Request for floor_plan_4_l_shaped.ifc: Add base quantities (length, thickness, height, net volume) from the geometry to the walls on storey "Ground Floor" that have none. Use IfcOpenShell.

First a look at what the model holds.

```python
import ifcopenshell
import ifcopenshell.util.element
import ifcopenshell.util.unit

model = ifcopenshell.open("floor_plan_4_l_shaped.ifc")
print(model.schema)
for unit_type in ("LENGTHUNIT", "AREAUNIT", "VOLUMEUNIT"):
    print(unit_type, ifcopenshell.util.unit.calculate_unit_scale(model, unit_type))
storey = next(s for s in model.by_type("IfcBuildingStorey") if s.Name == "Ground Floor")
walls = [e for e in ifcopenshell.util.element.get_decomposition(storey) if e.is_a("IfcWall")]
for e in sorted(walls, key=lambda e: e.id()):
    print(e.id(), e.is_a(), e.Name, list(ifcopenshell.util.element.get_psets(e, qtos_only=True)), sep=" | ")
```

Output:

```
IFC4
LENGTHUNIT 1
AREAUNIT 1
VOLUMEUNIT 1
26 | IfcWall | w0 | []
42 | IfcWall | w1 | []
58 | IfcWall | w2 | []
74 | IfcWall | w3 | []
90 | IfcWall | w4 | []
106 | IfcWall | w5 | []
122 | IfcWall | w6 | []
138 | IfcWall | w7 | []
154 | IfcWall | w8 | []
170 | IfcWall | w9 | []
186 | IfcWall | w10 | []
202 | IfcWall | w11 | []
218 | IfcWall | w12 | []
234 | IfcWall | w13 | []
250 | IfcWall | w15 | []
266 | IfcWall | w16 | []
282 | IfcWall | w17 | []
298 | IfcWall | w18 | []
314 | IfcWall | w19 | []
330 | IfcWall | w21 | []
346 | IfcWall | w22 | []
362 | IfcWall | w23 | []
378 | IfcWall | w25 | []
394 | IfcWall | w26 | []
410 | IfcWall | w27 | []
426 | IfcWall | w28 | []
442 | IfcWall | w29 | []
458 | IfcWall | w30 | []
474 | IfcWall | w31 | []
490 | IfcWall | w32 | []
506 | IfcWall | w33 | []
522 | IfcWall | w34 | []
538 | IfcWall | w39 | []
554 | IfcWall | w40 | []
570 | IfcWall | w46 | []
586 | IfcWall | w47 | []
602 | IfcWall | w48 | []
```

```python
import ifcopenshell
import ifcopenshell.api.pset
import ifcopenshell.geom
import ifcopenshell.util.element
import ifcopenshell.util.shape
import ifcopenshell.util.unit

model = ifcopenshell.open("floor_plan_4_l_shaped.ifc")
unit_scale = ifcopenshell.util.unit.calculate_unit_scale(model)
volume_scale = ifcopenshell.util.unit.calculate_unit_scale(model, "VOLUMEUNIT")
settings = ifcopenshell.geom.settings()

storey = next(s for s in model.by_type("IfcBuildingStorey") if s.Name == "Ground Floor")
walls = [e for e in ifcopenshell.util.element.get_decomposition(storey) if e.is_a("IfcWall")]

for e in sorted(walls, key=lambda e: e.id()):
    if ifcopenshell.util.element.get_psets(e, qtos_only=True, should_inherit=False):
        continue
    # Geometry comes back in metres, in the element's own axes.
    shape = ifcopenshell.geom.create_shape(settings, e)
    values = {
        "Length": ifcopenshell.util.shape.get_x(shape.geometry) / unit_scale,
        "Width": ifcopenshell.util.shape.get_y(shape.geometry) / unit_scale,
        "Height": ifcopenshell.util.shape.get_z(shape.geometry) / unit_scale,
        "NetVolume": ifcopenshell.util.shape.get_volume(shape.geometry) / volume_scale,
    }
    qto = ifcopenshell.api.pset.add_qto(model, product=e, name="Qto_WallBaseQuantities")
    ifcopenshell.api.pset.edit_qto(model, qto=qto, properties=values)
    print(e.id(), {k: round(v, 3) for k, v in values.items()})

model.write("floor_plan_4_l_shaped-out.ifc")
```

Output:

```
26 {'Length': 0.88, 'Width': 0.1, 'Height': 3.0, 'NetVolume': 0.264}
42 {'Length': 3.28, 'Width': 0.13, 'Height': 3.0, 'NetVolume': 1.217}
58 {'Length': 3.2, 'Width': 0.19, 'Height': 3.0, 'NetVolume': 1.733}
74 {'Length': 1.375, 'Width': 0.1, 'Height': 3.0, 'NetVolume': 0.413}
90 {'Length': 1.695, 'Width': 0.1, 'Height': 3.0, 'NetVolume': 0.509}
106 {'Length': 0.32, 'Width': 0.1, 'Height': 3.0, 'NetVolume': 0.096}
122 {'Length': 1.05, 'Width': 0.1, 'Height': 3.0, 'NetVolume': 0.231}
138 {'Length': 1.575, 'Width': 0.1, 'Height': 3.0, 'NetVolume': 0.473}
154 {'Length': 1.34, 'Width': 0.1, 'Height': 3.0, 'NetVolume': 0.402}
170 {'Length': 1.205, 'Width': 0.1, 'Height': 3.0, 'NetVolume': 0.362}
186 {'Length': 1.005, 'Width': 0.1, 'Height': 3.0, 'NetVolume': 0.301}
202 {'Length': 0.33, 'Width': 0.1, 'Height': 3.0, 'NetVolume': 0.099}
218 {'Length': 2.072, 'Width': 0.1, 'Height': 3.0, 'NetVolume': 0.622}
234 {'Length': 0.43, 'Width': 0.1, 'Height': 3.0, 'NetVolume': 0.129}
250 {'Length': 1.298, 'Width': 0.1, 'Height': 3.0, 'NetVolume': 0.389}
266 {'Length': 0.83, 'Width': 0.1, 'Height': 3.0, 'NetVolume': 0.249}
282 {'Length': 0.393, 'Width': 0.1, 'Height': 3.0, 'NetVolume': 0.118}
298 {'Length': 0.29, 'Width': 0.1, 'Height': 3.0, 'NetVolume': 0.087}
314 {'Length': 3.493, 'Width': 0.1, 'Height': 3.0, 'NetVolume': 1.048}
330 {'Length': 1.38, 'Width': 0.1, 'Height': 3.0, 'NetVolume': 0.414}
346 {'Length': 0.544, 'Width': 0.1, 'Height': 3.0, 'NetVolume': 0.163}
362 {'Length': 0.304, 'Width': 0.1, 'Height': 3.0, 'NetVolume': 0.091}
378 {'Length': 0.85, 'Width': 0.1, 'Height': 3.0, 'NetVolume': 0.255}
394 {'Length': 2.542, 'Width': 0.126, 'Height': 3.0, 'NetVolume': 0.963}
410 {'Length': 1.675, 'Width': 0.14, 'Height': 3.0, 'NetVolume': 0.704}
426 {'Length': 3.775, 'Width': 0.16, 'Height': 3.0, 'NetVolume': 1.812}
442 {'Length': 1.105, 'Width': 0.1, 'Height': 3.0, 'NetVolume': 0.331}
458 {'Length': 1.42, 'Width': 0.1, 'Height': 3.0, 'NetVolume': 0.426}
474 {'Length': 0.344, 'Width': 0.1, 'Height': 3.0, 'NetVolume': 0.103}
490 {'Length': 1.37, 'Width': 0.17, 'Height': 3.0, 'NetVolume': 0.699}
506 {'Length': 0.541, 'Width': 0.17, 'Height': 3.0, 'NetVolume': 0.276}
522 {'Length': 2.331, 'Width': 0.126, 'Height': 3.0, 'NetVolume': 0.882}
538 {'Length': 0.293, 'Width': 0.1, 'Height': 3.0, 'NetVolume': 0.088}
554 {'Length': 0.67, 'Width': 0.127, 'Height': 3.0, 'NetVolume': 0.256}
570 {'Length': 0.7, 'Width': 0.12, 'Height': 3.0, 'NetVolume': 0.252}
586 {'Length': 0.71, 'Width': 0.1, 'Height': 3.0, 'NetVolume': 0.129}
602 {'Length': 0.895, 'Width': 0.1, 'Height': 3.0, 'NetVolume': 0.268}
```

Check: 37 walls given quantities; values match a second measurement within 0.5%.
